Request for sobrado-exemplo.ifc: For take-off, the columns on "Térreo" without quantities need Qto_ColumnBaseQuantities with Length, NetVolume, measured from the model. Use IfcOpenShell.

First a look at what the model holds.

```python
import ifcopenshell
import ifcopenshell.util.element
import ifcopenshell.util.unit

model = ifcopenshell.open("sobrado-exemplo.ifc")
print(model.schema)
for unit_type in ("LENGTHUNIT", "AREAUNIT", "VOLUMEUNIT"):
    print(unit_type, ifcopenshell.util.unit.calculate_unit_scale(model, unit_type))
storey = next(s for s in model.by_type("IfcBuildingStorey") if s.Name == "Térreo")
columns = [e for e in ifcopenshell.util.element.get_decomposition(storey) if e.is_a("IfcColumn")]
for e in sorted(columns, key=lambda e: e.id()):
    print(e.id(), e.is_a(), e.Name, list(ifcopenshell.util.element.get_psets(e, qtos_only=True)), sep=" | ")
```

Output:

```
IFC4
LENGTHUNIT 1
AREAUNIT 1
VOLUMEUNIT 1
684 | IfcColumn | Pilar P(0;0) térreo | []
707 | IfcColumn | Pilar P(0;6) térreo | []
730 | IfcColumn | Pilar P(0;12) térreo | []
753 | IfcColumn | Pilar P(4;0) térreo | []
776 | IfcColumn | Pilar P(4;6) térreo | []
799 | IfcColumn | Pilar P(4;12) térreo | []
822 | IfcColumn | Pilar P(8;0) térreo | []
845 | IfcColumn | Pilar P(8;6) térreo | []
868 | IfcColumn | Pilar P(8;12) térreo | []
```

```python
import ifcopenshell
import ifcopenshell.api.pset
import ifcopenshell.geom
import ifcopenshell.util.element
import ifcopenshell.util.shape
import ifcopenshell.util.unit

model = ifcopenshell.open("sobrado-exemplo.ifc")
unit_scale = ifcopenshell.util.unit.calculate_unit_scale(model)
volume_scale = ifcopenshell.util.unit.calculate_unit_scale(model, "VOLUMEUNIT")
settings = ifcopenshell.geom.settings()

storey = next(s for s in model.by_type("IfcBuildingStorey") if s.Name == "Térreo")
columns = [e for e in ifcopenshell.util.element.get_decomposition(storey) if e.is_a("IfcColumn")]

for e in sorted(columns, key=lambda e: e.id()):
    if ifcopenshell.util.element.get_psets(e, qtos_only=True, should_inherit=False):
        continue
    # Geometry comes back in metres, in the element's own axes.
    shape = ifcopenshell.geom.create_shape(settings, e)
    values = {
        "Length": ifcopenshell.util.shape.get_z(shape.geometry) / unit_scale,
        "NetVolume": ifcopenshell.util.shape.get_volume(shape.geometry) / volume_scale,
    }
    qto = ifcopenshell.api.pset.add_qto(model, product=e, name="Qto_ColumnBaseQuantities")
    ifcopenshell.api.pset.edit_qto(model, qto=qto, properties=values)
    print(e.id(), {k: round(v, 3) for k, v in values.items()})

model.write("sobrado-exemplo_edited.ifc")
```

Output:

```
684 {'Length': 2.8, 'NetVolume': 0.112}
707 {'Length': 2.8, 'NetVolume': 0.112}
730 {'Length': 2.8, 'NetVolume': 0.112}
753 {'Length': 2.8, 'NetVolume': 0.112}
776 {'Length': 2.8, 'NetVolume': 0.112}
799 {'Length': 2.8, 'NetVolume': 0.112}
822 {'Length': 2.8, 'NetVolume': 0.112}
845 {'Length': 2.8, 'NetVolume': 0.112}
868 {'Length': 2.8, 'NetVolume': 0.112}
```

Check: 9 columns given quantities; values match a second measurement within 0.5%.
